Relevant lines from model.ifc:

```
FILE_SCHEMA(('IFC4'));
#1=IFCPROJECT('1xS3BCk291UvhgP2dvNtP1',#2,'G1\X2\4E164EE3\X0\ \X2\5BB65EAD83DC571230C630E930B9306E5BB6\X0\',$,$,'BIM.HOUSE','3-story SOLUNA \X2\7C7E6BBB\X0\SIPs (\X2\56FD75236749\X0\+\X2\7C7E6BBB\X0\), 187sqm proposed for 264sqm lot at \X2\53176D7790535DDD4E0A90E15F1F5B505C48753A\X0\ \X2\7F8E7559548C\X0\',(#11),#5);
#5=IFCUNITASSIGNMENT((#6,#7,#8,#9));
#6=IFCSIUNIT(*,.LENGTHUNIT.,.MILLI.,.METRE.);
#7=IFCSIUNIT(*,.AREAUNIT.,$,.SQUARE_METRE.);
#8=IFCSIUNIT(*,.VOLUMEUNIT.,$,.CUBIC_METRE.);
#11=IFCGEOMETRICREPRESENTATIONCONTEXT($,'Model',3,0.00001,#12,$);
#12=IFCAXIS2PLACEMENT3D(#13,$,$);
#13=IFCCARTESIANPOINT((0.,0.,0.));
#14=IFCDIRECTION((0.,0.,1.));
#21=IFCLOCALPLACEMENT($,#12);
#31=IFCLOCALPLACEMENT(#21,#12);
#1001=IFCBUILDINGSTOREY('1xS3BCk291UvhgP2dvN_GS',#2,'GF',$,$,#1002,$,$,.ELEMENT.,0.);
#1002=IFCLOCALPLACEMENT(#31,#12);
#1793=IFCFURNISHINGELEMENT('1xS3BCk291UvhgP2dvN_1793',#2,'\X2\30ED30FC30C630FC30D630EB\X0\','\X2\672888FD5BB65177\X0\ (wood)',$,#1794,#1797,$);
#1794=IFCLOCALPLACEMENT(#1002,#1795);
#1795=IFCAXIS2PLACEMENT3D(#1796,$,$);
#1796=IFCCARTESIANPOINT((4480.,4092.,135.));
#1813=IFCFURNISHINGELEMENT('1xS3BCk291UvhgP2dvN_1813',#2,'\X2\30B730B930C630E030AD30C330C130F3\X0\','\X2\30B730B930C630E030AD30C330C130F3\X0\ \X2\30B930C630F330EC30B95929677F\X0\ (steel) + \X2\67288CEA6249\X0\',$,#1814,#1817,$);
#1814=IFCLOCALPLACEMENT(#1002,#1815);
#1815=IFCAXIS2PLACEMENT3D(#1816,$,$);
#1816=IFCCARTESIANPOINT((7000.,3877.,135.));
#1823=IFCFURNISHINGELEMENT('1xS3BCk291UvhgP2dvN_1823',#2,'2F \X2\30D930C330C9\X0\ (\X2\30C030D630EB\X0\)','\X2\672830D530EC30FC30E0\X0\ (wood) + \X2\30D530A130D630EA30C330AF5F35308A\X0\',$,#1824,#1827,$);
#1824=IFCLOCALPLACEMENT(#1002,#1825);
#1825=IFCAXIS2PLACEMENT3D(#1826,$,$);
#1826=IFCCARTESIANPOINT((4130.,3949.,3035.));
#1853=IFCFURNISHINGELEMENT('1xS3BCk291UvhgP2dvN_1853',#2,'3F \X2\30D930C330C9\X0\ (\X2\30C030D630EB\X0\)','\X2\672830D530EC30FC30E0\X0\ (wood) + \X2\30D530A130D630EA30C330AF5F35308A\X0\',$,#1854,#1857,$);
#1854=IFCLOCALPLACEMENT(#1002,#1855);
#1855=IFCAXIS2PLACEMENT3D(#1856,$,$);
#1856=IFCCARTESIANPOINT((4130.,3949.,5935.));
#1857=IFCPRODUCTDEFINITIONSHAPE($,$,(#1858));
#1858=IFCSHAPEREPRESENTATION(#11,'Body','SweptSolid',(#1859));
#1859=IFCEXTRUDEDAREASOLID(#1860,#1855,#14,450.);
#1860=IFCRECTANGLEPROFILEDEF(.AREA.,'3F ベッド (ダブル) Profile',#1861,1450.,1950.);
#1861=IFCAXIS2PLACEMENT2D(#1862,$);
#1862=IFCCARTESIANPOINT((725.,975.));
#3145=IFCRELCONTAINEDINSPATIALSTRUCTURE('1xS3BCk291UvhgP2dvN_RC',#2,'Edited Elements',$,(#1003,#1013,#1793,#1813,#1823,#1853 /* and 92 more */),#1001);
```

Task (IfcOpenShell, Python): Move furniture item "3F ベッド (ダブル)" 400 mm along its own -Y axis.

```python
import ifcopenshell
import ifcopenshell.api.geometry
import ifcopenshell.util.placement
import ifcopenshell.util.unit

model = ifcopenshell.open("model.ifc")
unit_scale = ifcopenshell.util.unit.calculate_unit_scale(model)

item = model.by_guid("1xS3BCk291UvhgP2dvN_1853")
matrix = ifcopenshell.util.placement.get_local_placement(item.ObjectPlacement)
matrix[:3, 3] -= matrix[:3, 1] * 0.4 / unit_scale
ifcopenshell.api.geometry.edit_object_placement(model, product=item, matrix=matrix, is_si=False)

print(ifcopenshell.util.placement.get_local_placement(item.ObjectPlacement).round(3) + 0.0)

model.write("model-out.ifc")
```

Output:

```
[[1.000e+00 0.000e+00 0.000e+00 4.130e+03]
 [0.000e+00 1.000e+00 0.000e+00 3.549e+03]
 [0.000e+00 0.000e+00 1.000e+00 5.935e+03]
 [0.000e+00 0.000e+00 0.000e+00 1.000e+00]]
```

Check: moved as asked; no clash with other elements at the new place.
